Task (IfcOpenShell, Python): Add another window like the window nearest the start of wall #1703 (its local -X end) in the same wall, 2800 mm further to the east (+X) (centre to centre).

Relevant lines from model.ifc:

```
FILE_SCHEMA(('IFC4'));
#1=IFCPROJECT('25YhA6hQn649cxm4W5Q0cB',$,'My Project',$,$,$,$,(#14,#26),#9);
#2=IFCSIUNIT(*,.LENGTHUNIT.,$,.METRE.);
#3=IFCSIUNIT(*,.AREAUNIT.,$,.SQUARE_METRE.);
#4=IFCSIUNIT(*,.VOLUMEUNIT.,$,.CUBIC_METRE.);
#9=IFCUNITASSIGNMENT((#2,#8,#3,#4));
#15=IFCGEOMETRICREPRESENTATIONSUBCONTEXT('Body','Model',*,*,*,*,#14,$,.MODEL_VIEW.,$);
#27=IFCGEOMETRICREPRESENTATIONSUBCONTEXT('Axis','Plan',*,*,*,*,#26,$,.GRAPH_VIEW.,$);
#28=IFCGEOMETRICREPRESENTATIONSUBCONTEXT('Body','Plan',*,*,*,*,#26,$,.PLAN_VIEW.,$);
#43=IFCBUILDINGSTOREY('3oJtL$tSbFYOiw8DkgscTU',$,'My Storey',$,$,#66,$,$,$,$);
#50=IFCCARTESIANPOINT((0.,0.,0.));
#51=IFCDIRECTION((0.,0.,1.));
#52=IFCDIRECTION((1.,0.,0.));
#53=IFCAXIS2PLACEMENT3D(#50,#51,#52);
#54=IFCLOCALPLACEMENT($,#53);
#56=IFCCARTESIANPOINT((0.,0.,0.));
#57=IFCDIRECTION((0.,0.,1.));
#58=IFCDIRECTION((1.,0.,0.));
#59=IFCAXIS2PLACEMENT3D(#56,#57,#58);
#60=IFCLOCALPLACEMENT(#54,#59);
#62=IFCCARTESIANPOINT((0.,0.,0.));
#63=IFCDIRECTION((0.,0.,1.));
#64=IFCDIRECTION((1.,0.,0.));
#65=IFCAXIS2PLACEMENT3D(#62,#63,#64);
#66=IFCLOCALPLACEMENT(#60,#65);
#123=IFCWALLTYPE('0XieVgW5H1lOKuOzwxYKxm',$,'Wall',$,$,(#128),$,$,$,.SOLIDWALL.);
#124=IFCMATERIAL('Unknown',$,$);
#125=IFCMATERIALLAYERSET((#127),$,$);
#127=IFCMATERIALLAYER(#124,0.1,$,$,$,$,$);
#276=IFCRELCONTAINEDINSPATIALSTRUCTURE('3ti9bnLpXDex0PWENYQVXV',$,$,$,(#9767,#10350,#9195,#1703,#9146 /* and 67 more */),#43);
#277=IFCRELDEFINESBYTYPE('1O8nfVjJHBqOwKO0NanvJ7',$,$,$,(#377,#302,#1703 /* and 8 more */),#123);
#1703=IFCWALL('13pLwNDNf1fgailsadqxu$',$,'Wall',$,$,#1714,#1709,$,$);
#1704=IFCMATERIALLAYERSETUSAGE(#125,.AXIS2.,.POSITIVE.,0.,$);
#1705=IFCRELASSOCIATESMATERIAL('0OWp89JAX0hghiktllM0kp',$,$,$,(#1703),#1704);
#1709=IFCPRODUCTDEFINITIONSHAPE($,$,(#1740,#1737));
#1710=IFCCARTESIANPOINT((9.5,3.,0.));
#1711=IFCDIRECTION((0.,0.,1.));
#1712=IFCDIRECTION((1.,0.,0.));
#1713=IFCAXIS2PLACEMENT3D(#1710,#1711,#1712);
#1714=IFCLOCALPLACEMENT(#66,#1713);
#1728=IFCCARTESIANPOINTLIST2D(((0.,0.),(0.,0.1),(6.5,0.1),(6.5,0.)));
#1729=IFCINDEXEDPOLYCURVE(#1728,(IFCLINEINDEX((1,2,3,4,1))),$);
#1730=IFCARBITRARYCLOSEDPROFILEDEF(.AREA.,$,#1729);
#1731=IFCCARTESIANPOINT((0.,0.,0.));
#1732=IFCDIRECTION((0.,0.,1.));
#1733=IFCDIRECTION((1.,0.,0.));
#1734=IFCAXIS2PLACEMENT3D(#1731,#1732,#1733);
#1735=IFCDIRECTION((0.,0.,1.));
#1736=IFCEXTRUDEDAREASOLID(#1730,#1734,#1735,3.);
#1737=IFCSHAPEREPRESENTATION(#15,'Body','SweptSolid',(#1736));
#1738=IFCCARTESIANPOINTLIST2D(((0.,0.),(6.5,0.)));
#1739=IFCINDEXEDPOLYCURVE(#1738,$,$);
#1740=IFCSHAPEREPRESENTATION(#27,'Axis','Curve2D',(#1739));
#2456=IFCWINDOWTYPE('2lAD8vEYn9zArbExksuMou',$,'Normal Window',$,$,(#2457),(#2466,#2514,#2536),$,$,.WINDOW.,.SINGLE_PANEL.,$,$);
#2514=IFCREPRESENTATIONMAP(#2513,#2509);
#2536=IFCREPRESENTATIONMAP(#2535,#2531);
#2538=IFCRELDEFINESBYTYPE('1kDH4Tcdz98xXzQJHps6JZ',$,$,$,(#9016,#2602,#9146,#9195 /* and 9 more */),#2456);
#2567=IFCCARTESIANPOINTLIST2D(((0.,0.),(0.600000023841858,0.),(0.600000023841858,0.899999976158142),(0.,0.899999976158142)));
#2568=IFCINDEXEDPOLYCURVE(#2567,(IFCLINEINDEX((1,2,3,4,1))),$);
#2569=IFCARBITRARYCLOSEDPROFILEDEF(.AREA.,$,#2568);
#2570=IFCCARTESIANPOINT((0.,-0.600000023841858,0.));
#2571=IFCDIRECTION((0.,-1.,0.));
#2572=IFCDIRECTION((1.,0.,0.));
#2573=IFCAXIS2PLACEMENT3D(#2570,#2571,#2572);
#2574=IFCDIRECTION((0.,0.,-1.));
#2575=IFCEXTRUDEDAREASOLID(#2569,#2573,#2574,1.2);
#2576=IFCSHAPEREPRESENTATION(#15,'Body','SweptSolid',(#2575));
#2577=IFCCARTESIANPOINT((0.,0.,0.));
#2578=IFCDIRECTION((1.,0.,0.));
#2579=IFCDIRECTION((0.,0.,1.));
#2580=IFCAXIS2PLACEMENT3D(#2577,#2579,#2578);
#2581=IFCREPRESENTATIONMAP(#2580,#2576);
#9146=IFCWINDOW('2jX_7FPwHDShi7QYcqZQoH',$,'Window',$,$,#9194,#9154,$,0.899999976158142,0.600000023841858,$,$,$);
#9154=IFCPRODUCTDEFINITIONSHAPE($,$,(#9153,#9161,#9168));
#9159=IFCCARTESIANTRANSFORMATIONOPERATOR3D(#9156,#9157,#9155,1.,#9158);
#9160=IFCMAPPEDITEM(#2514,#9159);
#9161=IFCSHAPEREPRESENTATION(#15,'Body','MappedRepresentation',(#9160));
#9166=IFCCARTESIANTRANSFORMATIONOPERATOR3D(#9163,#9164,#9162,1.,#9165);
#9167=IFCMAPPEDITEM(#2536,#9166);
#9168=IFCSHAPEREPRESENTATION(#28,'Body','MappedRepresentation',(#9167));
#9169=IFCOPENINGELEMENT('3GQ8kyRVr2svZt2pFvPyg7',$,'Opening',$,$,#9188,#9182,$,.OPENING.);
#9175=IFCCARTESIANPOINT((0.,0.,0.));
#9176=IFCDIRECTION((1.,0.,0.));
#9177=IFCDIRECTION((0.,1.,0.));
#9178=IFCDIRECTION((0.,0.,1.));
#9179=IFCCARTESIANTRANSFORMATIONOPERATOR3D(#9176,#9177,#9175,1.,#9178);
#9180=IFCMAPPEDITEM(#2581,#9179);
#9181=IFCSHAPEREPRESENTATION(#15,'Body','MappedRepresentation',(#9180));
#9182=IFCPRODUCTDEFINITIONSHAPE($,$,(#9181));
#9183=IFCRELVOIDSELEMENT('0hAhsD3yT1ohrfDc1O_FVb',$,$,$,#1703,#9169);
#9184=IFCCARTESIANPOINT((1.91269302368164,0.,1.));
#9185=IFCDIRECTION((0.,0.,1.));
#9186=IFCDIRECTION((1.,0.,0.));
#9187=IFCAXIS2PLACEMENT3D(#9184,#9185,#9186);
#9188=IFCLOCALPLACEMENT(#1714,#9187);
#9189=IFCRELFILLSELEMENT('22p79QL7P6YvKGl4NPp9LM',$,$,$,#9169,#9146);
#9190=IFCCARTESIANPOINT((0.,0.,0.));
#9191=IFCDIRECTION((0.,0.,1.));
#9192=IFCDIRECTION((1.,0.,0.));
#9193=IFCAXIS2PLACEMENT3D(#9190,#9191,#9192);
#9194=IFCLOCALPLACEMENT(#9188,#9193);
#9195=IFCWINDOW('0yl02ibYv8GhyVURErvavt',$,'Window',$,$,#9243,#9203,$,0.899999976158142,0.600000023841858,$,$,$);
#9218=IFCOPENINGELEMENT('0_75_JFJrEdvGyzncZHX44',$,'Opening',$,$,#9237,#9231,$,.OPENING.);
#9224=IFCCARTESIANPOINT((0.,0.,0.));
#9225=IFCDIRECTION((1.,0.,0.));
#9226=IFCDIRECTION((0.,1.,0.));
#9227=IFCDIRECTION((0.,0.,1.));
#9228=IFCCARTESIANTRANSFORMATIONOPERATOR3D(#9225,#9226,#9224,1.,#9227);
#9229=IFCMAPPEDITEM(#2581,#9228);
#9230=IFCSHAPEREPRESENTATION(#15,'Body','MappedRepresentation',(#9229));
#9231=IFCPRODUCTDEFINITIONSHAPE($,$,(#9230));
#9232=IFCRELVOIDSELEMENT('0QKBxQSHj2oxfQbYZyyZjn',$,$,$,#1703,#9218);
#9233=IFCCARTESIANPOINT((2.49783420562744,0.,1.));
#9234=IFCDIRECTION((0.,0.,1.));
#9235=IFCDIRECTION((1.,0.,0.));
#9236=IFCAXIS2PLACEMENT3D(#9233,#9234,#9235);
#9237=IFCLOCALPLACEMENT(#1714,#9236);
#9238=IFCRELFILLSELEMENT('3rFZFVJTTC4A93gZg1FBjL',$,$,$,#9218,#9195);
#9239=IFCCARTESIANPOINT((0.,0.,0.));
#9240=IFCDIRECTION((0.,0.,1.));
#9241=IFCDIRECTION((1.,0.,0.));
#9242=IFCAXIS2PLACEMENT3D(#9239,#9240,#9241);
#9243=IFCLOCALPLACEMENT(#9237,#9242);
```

```python
import ifcopenshell
import ifcopenshell.api.feature
import ifcopenshell.api.geometry
import ifcopenshell.api.root
import ifcopenshell.geom
import ifcopenshell.util.element
import ifcopenshell.util.placement
import ifcopenshell.util.shape
import ifcopenshell.util.unit

model = ifcopenshell.open("model.ifc")
unit_scale = ifcopenshell.util.unit.calculate_unit_scale(model)
settings = ifcopenshell.geom.settings()


def volume(element):
    """Net volume in cubic metres, openings subtracted."""
    shape = ifcopenshell.geom.create_shape(settings, element)
    return ifcopenshell.util.shape.get_volume(shape.geometry)


window = model.by_guid("2jX_7FPwHDShi7QYcqZQoH")
opening = window.FillsVoids[0].RelatingOpeningElement
wall = opening.VoidsElements[0].RelatingBuildingElement
before = volume(wall)
shift = ifcopenshell.util.placement.get_local_placement(wall.ObjectPlacement)[:3, 0] * 2.8 / unit_scale

# copy_class copies the void relationship, type, container and properties, but no geometry.
new_opening = ifcopenshell.api.root.copy_class(model, product=opening)
new_opening.Representation = ifcopenshell.util.element.copy_deep(
    model, opening.Representation, exclude=["IfcGeometricRepresentationContext", "IfcRepresentationMap"]
)
new_window = ifcopenshell.api.root.copy_class(model, product=window)
new_window.Representation = ifcopenshell.util.element.copy_deep(
    model, window.Representation, exclude=["IfcGeometricRepresentationContext", "IfcRepresentationMap"]
)
ifcopenshell.api.feature.add_filling(model, opening=new_opening, element=new_window)

for old, new in ((opening, new_opening), (window, new_window)):
    matrix = ifcopenshell.util.placement.get_local_placement(old.ObjectPlacement)
    matrix[:3, 3] += shift
    ifcopenshell.api.geometry.edit_object_placement(model, product=new, matrix=matrix, is_si=False)

after = volume(wall)

print(f"wall volume {before:.3f} -> {after:.3f} m3")

model.write("model_edited.ifc")
```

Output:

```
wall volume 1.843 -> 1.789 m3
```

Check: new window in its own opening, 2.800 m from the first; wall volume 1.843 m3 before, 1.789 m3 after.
